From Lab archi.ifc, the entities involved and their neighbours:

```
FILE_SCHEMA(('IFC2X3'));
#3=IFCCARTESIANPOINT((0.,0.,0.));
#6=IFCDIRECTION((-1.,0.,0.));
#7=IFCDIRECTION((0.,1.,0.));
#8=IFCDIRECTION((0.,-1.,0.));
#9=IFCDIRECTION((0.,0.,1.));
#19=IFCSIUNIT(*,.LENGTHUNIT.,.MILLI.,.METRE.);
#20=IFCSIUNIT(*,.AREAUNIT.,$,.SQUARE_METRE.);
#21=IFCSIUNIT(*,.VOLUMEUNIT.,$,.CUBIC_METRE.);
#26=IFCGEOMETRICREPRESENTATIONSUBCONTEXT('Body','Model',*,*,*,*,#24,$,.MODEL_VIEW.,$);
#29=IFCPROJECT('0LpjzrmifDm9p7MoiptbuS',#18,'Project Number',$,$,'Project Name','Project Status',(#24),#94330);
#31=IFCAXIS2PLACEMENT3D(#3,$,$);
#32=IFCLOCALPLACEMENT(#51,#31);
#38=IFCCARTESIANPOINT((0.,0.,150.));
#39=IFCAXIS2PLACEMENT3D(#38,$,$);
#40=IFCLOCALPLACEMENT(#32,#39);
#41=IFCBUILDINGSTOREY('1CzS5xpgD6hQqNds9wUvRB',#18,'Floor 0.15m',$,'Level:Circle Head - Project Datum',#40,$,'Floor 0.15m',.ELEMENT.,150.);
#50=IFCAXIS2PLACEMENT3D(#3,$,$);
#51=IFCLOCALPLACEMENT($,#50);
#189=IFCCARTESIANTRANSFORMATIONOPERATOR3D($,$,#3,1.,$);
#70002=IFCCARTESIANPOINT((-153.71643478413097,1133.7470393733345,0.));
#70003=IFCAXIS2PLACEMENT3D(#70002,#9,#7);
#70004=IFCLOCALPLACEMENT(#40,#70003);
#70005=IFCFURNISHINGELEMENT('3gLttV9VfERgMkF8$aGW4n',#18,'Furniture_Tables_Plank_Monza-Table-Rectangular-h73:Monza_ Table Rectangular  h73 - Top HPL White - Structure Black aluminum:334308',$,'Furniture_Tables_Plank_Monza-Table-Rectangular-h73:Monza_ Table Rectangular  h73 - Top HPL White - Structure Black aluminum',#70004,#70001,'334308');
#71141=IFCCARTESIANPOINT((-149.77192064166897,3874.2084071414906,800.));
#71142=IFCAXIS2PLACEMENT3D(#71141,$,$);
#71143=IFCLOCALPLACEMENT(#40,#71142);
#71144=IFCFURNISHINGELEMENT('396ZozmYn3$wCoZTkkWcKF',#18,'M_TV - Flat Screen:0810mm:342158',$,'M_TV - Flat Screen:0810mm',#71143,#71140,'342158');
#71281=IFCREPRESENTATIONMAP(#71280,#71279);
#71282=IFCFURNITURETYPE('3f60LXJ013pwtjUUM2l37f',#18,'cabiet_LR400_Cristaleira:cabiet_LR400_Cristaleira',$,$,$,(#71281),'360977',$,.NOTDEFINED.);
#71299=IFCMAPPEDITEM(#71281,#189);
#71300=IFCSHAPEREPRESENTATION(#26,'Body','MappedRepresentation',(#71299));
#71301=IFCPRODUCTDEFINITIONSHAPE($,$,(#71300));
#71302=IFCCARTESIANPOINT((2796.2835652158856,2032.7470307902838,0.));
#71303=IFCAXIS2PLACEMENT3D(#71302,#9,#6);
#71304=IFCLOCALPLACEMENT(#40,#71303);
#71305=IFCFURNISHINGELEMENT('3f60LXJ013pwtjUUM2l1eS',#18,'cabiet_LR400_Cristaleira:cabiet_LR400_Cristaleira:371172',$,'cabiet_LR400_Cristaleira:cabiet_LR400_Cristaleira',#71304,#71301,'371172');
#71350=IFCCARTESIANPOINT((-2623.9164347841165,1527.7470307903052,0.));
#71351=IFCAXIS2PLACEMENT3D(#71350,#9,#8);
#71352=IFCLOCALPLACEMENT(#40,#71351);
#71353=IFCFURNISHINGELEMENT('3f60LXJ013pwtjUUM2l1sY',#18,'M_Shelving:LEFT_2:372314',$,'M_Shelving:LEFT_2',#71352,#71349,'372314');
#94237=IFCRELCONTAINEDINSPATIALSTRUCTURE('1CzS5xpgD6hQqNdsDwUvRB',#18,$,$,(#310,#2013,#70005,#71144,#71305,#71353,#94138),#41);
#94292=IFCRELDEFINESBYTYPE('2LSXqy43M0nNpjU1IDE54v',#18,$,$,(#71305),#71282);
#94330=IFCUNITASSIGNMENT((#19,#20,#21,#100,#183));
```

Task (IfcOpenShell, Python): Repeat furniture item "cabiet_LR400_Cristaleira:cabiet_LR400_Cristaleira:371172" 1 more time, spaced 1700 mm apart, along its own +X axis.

```python
import ifcopenshell
import ifcopenshell.api.geometry
import ifcopenshell.api.root
import ifcopenshell.util.element
import ifcopenshell.util.placement

model = ifcopenshell.open("Lab archi.ifc")


def reuse_history(source, copy):
    """copy_class also copies each property set's owner history, people and application; keep the originals."""
    for rel in copy.IsDefinedBy:
        if rel.is_a("IfcRelDefinesByProperties") and (history := rel.RelatingPropertyDefinition.OwnerHistory):
            rel.RelatingPropertyDefinition.OwnerHistory = source.OwnerHistory
            ifcopenshell.util.element.remove_deep2(model, history)


source = model.by_id(71305)
base = ifcopenshell.util.placement.get_local_placement(source.ObjectPlacement)
step = base[:3, 0] * 1700.0

for i in range(1, 2):
    copy = ifcopenshell.api.root.copy_class(model, product=source)
    copy.Representation = ifcopenshell.util.element.copy_deep(
        model, source.Representation, exclude=["IfcGeometricRepresentationContext", "IfcRepresentationMap"]
    )
    copy.Name = "cabiet_LR400_Cristaleira:cabiet_LR400_Cristaleira"
    copy.Tag = None
    reuse_history(source, copy)
    matrix = base.copy()
    matrix[:3, 3] += i * step
    print("added at", matrix[:3, 3].round(3) + 0.0)
    ifcopenshell.api.geometry.edit_object_placement(model, product=copy, matrix=matrix, is_si=False)

model.write("Lab archi-out.ifc")
```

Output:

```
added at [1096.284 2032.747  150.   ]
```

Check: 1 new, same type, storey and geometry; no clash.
